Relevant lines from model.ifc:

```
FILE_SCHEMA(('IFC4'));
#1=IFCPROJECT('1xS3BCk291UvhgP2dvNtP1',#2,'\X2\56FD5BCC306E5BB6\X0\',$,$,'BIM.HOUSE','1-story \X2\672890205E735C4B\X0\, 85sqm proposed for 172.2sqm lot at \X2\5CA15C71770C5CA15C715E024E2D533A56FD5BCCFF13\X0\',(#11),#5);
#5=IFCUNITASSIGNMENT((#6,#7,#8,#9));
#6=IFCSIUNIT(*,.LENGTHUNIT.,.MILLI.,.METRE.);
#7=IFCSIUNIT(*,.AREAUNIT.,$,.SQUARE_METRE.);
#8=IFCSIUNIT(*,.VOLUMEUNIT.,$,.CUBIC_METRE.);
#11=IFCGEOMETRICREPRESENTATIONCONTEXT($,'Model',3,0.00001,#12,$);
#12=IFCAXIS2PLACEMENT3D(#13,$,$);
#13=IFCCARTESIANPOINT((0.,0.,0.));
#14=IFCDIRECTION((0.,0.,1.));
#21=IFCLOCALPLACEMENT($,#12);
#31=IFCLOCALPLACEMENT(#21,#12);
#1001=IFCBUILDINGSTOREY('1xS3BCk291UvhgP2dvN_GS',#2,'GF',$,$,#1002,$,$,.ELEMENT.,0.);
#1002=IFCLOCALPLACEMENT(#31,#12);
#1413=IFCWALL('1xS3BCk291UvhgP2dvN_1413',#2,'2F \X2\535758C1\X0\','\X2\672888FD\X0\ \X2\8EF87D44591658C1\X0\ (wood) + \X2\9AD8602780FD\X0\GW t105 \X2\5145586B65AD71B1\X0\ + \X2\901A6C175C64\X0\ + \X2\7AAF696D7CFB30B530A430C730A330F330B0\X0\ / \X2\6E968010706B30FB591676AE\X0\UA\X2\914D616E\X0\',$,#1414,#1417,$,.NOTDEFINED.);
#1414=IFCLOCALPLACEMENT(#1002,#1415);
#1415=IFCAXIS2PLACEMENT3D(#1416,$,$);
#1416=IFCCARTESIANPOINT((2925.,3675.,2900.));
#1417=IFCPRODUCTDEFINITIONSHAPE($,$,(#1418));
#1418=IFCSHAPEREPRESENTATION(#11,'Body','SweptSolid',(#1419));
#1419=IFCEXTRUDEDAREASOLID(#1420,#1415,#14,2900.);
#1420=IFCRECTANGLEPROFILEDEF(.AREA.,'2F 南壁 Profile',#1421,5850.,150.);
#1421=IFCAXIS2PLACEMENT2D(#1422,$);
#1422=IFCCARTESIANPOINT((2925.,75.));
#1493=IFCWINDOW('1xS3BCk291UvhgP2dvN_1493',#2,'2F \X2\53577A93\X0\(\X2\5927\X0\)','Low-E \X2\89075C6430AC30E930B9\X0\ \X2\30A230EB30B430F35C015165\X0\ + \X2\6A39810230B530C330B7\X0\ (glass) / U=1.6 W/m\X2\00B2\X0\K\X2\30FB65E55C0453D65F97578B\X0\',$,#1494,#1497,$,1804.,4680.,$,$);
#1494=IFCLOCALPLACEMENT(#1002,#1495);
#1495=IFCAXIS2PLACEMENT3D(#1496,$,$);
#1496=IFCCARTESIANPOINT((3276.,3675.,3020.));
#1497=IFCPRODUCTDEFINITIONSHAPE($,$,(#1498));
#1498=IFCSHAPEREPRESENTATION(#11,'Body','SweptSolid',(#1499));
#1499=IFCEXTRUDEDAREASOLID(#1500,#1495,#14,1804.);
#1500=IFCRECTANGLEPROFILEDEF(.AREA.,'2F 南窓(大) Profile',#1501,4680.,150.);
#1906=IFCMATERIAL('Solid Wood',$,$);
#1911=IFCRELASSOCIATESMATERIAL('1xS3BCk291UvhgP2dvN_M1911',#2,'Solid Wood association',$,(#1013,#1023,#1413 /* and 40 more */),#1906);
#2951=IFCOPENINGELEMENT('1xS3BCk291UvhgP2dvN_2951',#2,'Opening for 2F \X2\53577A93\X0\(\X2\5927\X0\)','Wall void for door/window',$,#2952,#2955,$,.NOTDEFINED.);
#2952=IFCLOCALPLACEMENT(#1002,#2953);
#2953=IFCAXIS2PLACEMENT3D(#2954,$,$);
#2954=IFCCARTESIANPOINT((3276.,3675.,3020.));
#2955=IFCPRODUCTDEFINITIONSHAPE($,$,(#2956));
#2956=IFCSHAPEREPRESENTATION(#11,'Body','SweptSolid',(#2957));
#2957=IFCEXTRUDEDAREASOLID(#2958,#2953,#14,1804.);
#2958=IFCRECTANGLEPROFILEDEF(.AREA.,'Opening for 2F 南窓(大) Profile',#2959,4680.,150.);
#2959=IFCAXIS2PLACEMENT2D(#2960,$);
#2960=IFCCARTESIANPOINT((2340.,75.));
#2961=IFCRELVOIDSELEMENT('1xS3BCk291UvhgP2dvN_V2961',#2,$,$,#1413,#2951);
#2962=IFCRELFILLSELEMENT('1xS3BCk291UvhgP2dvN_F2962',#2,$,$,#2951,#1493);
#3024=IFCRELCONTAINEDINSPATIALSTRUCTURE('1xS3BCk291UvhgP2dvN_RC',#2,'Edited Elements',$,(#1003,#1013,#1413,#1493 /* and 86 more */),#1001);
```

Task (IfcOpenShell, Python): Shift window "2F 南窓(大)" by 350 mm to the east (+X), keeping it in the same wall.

```python
import ifcopenshell
import ifcopenshell.api.geometry
import ifcopenshell.util.placement
import ifcopenshell.util.unit

model = ifcopenshell.open("model.ifc")
unit_scale = ifcopenshell.util.unit.calculate_unit_scale(model)

window = model.by_id(1493)
opening = window.FillsVoids[0].RelatingOpeningElement
wall = opening.VoidsElements[0].RelatingBuildingElement

wall_matrix = ifcopenshell.util.placement.get_local_placement(wall.ObjectPlacement)
shift = wall_matrix[:3, 0] * 0.35 / unit_scale
before = ifcopenshell.util.placement.get_local_placement(window.ObjectPlacement)[:3, 3].copy()

# The window is not placed relative to its opening, so move both.
for product in (opening, window):
    matrix = ifcopenshell.util.placement.get_local_placement(product.ObjectPlacement)
    matrix[:3, 3] += shift
    ifcopenshell.api.geometry.edit_object_placement(model, product=product, matrix=matrix, is_si=False)

after = ifcopenshell.util.placement.get_local_placement(window.ObjectPlacement)[:3, 3]
print("window moved by", (after - before).round(3) + 0.0)

model.write("model_v2.ifc")
```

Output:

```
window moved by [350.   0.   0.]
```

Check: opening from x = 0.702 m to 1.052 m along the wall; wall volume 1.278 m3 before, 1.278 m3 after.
